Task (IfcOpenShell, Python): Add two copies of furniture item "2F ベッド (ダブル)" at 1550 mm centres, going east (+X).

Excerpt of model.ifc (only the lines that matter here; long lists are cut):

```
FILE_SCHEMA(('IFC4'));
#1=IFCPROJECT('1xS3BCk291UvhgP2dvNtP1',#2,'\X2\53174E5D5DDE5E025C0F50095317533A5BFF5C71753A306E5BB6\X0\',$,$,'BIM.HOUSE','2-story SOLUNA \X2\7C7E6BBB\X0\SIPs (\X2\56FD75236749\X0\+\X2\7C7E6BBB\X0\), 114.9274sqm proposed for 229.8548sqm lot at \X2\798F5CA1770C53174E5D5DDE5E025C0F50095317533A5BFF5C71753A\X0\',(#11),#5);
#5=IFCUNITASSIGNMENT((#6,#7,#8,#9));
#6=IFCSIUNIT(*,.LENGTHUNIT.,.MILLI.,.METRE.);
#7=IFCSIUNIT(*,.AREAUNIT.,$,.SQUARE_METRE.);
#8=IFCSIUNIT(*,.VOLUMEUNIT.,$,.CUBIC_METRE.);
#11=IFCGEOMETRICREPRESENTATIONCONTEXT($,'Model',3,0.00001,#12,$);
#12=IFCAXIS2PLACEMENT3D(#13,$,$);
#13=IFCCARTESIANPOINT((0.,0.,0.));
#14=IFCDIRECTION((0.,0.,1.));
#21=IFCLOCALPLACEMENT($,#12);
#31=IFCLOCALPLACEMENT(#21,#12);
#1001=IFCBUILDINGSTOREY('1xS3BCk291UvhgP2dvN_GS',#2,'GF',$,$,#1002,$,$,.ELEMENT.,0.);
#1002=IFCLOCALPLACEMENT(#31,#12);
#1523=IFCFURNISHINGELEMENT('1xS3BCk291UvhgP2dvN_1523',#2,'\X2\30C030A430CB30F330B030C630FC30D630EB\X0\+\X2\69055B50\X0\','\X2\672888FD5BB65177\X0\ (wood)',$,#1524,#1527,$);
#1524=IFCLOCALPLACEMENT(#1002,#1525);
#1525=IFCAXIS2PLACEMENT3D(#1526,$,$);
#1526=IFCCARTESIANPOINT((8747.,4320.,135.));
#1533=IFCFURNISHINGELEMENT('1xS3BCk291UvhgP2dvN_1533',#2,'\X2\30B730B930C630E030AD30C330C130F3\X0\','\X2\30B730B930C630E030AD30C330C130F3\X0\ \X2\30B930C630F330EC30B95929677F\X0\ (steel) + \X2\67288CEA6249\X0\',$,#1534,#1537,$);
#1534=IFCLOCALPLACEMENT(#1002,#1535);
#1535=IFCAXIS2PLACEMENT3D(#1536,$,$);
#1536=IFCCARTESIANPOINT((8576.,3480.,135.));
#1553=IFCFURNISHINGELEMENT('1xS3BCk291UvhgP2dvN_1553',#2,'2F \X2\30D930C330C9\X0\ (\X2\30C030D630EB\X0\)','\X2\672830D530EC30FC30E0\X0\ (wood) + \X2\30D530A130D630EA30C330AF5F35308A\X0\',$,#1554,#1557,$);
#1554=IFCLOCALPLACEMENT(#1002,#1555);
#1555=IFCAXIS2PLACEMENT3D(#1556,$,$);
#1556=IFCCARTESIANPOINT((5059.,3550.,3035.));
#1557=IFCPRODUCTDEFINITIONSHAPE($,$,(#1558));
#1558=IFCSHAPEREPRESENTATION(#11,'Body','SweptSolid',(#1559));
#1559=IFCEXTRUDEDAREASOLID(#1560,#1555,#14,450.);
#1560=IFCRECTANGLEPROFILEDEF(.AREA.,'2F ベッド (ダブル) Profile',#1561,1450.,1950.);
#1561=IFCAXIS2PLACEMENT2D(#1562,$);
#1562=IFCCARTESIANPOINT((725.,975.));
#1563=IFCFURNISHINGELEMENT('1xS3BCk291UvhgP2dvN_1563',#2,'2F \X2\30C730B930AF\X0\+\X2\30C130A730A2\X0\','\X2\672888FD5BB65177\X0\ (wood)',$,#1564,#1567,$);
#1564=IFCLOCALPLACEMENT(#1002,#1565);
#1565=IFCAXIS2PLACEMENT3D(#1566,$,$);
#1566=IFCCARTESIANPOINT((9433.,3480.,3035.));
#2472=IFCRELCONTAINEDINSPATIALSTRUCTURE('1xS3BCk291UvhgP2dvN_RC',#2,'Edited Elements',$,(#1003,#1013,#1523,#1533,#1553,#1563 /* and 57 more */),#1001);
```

```python
import numpy as np
import ifcopenshell
import ifcopenshell.api.geometry
import ifcopenshell.api.root
import ifcopenshell.util.element
import ifcopenshell.util.placement

model = ifcopenshell.open("model.ifc")


def reuse_history(source, copy):
    """copy_class also copies each property set's owner history, people and application; keep the originals."""
    for rel in copy.IsDefinedBy:
        if rel.is_a("IfcRelDefinesByProperties") and (history := rel.RelatingPropertyDefinition.OwnerHistory):
            rel.RelatingPropertyDefinition.OwnerHistory = source.OwnerHistory
            ifcopenshell.util.element.remove_deep2(model, history)


source = model.by_guid("1xS3BCk291UvhgP2dvN_1553")
base = ifcopenshell.util.placement.get_local_placement(source.ObjectPlacement)
step = np.array([1.0, 0.0, 0.0]) * 1550.0

for i in range(1, 3):
    copy = ifcopenshell.api.root.copy_class(model, product=source)
    copy.Representation = ifcopenshell.util.element.copy_deep(
        model, source.Representation, exclude=["IfcGeometricRepresentationContext", "IfcRepresentationMap"]
    )
    reuse_history(source, copy)
    matrix = base.copy()
    matrix[:3, 3] += i * step
    print("added at", matrix[:3, 3].round(3) + 0.0)
    ifcopenshell.api.geometry.edit_object_placement(model, product=copy, matrix=matrix, is_si=False)

model.write("model_edited.ifc")
```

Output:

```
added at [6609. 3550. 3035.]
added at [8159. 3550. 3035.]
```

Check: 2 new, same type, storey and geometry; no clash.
